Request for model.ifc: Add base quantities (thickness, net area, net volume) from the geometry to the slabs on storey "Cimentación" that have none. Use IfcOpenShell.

First a look at what the model holds.

```python
import ifcopenshell
import ifcopenshell.util.element
import ifcopenshell.util.unit

model = ifcopenshell.open("model.ifc")
print(model.schema)
for unit_type in ("LENGTHUNIT", "AREAUNIT", "VOLUMEUNIT"):
    print(unit_type, ifcopenshell.util.unit.calculate_unit_scale(model, unit_type))
storey = next(s for s in model.by_type("IfcBuildingStorey") if s.Name == "Cimentación")
slabs = [e for e in ifcopenshell.util.element.get_decomposition(storey) if e.is_a("IfcSlab")]
for e in sorted(slabs, key=lambda e: e.id()):
    print(e.id(), e.is_a(), e.Name, list(ifcopenshell.util.element.get_psets(e, qtos_only=True)), sep=" | ")
```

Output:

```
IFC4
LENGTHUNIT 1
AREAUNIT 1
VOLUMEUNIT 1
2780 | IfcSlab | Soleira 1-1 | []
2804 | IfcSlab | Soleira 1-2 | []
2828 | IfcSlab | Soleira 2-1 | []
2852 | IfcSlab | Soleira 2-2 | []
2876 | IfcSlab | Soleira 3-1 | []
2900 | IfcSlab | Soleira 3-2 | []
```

```python
import ifcopenshell
import ifcopenshell.api.pset
import ifcopenshell.geom
import ifcopenshell.util.element
import ifcopenshell.util.shape
import ifcopenshell.util.unit

model = ifcopenshell.open("model.ifc")
unit_scale = ifcopenshell.util.unit.calculate_unit_scale(model)
area_scale = ifcopenshell.util.unit.calculate_unit_scale(model, "AREAUNIT")
volume_scale = ifcopenshell.util.unit.calculate_unit_scale(model, "VOLUMEUNIT")
settings = ifcopenshell.geom.settings()

storey = next(s for s in model.by_type("IfcBuildingStorey") if s.Name == "Cimentación")
slabs = [e for e in ifcopenshell.util.element.get_decomposition(storey) if e.is_a("IfcSlab")]

for e in sorted(slabs, key=lambda e: e.id()):
    if ifcopenshell.util.element.get_psets(e, qtos_only=True, should_inherit=False):
        continue
    # Geometry comes back in metres, in the element's own axes.
    shape = ifcopenshell.geom.create_shape(settings, e)
    values = {
        "Width": ifcopenshell.util.shape.get_z(shape.geometry) / unit_scale,
        "NetArea": ifcopenshell.util.shape.get_footprint_area(shape.geometry) / area_scale,
        "NetVolume": ifcopenshell.util.shape.get_volume(shape.geometry) / volume_scale,
    }
    qto = ifcopenshell.api.pset.add_qto(model, product=e, name="Qto_SlabBaseQuantities")
    ifcopenshell.api.pset.edit_qto(model, qto=qto, properties=values)
    print(e.id(), {k: round(v, 3) for k, v in values.items()})

model.write("model_updated.ifc")
```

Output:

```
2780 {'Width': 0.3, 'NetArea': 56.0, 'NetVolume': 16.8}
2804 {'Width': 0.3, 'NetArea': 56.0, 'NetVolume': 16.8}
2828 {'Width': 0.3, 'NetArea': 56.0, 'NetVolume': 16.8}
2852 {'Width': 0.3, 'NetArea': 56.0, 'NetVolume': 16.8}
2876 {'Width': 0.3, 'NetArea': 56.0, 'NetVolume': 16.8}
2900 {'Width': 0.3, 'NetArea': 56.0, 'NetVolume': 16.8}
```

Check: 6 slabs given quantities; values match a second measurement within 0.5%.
